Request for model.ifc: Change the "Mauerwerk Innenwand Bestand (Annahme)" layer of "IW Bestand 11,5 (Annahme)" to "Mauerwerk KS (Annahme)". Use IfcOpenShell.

First a look at what the model holds.

```python
import ifcopenshell
import ifcopenshell.util.element

model = ifcopenshell.open("model.ifc")
print(model.schema)
for layer_set in model.by_type("IfcMaterialLayerSet"):
    if layer_set.LayerSetName == "IW Bestand 11,5 (Annahme)":
        for layer in layer_set.MaterialLayers:
            print(layer.id(), layer.Material and layer.Material.Name, layer.LayerThickness, sep=" | ")
        print(len(ifcopenshell.util.element.get_elements_by_material(model, layer_set)), "elements and types use it")
print(sorted(m.Name for m in model.by_type("IfcMaterial") if m.Name)[:60])
```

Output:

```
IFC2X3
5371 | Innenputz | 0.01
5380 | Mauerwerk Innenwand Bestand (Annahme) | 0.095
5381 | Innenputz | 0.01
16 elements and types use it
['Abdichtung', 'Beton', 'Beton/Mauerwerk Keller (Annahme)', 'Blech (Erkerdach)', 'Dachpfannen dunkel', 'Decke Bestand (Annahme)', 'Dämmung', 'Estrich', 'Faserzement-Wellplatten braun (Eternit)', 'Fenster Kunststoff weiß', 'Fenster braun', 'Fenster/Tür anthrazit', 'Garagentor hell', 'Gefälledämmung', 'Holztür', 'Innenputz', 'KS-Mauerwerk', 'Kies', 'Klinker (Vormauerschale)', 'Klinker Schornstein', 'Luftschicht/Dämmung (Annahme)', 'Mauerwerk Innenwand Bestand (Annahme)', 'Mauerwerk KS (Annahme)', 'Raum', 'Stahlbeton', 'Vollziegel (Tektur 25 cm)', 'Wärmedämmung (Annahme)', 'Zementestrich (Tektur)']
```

```python
import ifcopenshell
import ifcopenshell.api.material

model = ifcopenshell.open("model.ifc")

layer_set = next(s for s in model.by_type("IfcMaterialLayerSet") if s.LayerSetName == "IW Bestand 11,5 (Annahme)")
layer = next(l for l in layer_set.MaterialLayers if l.Material and l.Material.Name == "Mauerwerk Innenwand Bestand (Annahme)")
material = next(m for m in model.by_type("IfcMaterial") if m.Name == "Mauerwerk KS (Annahme)")

# Point this one layer at the other material; renaming the old one would change it everywhere.
ifcopenshell.api.material.edit_layer(model, layer=layer, attributes={}, material=material)

print([l.Material.Name if l.Material else None for l in layer_set.MaterialLayers])

model.write("model_rev.ifc")
```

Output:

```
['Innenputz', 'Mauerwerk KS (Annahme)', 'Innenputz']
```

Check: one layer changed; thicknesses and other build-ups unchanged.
